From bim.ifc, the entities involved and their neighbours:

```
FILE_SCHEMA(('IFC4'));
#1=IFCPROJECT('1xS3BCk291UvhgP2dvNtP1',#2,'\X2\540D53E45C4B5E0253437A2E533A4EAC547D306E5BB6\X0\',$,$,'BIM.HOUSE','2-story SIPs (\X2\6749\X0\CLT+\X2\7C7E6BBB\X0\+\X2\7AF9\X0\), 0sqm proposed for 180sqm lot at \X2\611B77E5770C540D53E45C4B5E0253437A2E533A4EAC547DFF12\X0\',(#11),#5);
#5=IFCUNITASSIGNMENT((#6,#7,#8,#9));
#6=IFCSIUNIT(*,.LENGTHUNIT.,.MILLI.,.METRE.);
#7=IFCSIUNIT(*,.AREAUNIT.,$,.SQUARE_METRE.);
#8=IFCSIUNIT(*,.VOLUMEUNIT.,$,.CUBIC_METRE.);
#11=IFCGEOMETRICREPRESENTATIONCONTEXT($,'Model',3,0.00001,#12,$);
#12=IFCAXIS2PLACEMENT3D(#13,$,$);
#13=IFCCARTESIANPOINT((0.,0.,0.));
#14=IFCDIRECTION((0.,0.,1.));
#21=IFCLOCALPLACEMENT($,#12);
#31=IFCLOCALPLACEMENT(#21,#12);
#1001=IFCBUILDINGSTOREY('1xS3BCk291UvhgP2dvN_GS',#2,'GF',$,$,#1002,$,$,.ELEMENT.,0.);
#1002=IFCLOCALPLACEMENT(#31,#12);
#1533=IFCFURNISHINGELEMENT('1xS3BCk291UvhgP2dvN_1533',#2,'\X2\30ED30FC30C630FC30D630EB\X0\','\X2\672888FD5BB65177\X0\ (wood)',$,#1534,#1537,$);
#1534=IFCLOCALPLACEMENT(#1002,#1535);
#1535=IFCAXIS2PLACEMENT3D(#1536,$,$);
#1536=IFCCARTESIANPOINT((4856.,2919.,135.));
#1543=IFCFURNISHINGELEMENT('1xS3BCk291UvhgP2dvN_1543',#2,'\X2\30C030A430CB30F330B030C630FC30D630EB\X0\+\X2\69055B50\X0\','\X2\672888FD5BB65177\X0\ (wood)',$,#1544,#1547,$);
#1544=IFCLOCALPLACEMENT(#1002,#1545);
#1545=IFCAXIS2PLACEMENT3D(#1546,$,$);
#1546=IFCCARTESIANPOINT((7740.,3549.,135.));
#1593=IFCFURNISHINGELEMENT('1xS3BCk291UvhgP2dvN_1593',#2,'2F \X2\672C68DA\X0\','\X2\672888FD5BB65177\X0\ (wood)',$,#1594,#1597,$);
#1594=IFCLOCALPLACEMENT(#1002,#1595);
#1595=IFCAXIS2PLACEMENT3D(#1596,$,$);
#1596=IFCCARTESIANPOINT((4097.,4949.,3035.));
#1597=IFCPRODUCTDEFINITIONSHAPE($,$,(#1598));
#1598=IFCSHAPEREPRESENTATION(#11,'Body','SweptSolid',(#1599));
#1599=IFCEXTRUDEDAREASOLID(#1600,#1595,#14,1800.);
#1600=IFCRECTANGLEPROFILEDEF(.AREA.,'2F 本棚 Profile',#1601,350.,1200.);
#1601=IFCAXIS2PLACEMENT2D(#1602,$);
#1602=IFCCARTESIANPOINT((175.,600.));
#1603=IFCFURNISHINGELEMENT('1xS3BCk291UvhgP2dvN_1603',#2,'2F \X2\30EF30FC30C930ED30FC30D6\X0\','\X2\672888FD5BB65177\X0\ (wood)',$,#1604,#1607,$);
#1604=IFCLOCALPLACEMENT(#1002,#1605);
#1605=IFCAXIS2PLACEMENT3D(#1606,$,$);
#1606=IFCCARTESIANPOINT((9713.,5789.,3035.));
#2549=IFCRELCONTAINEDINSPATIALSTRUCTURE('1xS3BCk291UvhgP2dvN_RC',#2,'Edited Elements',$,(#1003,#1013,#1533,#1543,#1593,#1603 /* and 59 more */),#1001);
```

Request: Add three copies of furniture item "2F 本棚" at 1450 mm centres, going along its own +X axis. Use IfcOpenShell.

```python
import ifcopenshell
import ifcopenshell.api.geometry
import ifcopenshell.api.root
import ifcopenshell.util.element
import ifcopenshell.util.placement
import ifcopenshell.util.unit

model = ifcopenshell.open("bim.ifc")
unit_scale = ifcopenshell.util.unit.calculate_unit_scale(model)


def reuse_history(source, copy):
    """copy_class also copies each property set's owner history, people and application; keep the originals."""
    for rel in copy.IsDefinedBy:
        if rel.is_a("IfcRelDefinesByProperties") and (history := rel.RelatingPropertyDefinition.OwnerHistory):
            rel.RelatingPropertyDefinition.OwnerHistory = source.OwnerHistory
            ifcopenshell.util.element.remove_deep2(model, history)


source = model.by_guid("1xS3BCk291UvhgP2dvN_1593")
base = ifcopenshell.util.placement.get_local_placement(source.ObjectPlacement)
step = base[:3, 0] * 1.45 / unit_scale

for i in range(1, 4):
    copy = ifcopenshell.api.root.copy_class(model, product=source)
    copy.Representation = ifcopenshell.util.element.copy_deep(
        model, source.Representation, exclude=["IfcGeometricRepresentationContext", "IfcRepresentationMap"]
    )
    reuse_history(source, copy)
    matrix = base.copy()
    matrix[:3, 3] += i * step
    print("added at", matrix[:3, 3].round(3) + 0.0)
    ifcopenshell.api.geometry.edit_object_placement(model, product=copy, matrix=matrix, is_si=False)

model.write("bim-out.ifc")
```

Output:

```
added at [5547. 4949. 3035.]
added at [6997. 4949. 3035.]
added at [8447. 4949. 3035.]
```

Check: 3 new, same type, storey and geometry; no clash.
